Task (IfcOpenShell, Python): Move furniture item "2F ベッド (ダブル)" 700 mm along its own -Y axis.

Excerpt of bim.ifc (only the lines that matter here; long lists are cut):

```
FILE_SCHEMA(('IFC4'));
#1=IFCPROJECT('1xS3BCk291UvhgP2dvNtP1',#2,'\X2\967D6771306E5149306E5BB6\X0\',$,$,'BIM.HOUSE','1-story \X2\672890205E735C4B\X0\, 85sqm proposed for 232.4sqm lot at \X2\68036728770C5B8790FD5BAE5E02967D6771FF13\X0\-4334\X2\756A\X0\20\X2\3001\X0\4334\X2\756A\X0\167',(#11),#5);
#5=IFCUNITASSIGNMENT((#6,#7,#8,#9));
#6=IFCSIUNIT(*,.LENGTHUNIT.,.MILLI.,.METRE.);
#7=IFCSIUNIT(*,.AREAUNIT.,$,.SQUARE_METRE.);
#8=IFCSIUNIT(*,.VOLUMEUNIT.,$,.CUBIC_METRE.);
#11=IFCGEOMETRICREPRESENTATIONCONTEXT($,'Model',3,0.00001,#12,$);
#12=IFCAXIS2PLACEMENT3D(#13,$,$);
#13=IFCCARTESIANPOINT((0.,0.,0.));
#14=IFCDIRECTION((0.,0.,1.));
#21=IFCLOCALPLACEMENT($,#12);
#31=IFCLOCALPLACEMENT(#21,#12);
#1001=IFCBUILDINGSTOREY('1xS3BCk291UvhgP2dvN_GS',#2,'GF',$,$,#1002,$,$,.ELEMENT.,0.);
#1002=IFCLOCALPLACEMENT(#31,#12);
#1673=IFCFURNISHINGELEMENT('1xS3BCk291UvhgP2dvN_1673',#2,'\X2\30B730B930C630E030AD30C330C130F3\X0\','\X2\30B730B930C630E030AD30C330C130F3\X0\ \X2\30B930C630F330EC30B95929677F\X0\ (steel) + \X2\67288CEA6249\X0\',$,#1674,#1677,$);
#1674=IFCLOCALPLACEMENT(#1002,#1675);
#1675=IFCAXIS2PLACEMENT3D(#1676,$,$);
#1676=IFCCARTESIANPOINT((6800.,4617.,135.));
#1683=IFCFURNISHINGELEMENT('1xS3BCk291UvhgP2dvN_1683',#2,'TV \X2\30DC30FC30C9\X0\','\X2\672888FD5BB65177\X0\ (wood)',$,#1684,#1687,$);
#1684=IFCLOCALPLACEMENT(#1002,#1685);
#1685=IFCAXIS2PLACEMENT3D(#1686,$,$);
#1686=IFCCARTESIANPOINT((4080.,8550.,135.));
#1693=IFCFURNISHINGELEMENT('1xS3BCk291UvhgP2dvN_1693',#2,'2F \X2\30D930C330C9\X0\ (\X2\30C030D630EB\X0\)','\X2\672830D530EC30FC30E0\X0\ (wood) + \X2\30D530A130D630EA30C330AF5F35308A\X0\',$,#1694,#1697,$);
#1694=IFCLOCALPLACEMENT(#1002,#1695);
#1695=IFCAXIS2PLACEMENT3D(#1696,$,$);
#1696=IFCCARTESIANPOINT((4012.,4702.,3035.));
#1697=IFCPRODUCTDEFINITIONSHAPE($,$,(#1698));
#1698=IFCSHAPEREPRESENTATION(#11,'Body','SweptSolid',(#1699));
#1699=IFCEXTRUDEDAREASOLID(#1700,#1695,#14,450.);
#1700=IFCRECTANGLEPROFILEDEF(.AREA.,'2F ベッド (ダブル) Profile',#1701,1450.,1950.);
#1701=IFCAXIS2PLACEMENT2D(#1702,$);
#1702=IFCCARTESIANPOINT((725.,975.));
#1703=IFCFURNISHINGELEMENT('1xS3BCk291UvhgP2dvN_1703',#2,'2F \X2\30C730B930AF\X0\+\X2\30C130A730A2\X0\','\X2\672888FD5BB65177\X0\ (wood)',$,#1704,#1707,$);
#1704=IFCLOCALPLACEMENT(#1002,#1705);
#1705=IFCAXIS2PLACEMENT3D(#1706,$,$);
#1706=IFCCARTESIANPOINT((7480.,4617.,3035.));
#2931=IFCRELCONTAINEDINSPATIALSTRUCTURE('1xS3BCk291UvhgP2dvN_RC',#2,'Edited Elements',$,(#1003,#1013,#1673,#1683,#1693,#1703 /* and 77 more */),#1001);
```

```python
import ifcopenshell
import ifcopenshell.api.geometry
import ifcopenshell.util.placement

model = ifcopenshell.open("bim.ifc")

item = model.by_id(1693)
matrix = ifcopenshell.util.placement.get_local_placement(item.ObjectPlacement)
matrix[:3, 3] -= matrix[:3, 1] * 700.0
ifcopenshell.api.geometry.edit_object_placement(model, product=item, matrix=matrix, is_si=False)

print(ifcopenshell.util.placement.get_local_placement(item.ObjectPlacement).round(3) + 0.0)

model.write("bim_rev.ifc")
```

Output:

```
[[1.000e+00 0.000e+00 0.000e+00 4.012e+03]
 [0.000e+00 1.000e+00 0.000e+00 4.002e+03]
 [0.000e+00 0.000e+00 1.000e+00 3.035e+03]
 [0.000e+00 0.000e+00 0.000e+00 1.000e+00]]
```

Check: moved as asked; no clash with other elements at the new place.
